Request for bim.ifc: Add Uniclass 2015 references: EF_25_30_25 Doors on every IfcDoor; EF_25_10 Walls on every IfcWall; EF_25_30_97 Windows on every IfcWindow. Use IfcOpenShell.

First a look at what the model holds.

```python
import ifcopenshell

model = ifcopenshell.open("bim.ifc")
print(model.schema)
print("classifications:", [c.Name for c in model.by_type("IfcClassification")])
for ifc_class in ("IfcDoor", "IfcRoof", "IfcStair", "IfcWall", "IfcWindow"):
    print(ifc_class, len(model.by_type(ifc_class)))
```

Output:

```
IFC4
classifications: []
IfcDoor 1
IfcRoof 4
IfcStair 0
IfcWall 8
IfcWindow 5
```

```python
import ifcopenshell
import ifcopenshell.api.classification

model = ifcopenshell.open("bim.ifc")

system = ifcopenshell.api.classification.add_classification(model, classification="Uniclass 2015")

codes = {
    "IfcDoor": ("EF_25_30_25", "Doors"),
    "IfcWall": ("EF_25_10", "Walls"),
    "IfcWindow": ("EF_25_30_97", "Windows"),
}
for ifc_class, (code, name) in codes.items():
    products = model.by_type(ifc_class)
    ifcopenshell.api.classification.add_reference(
        model, products=products, classification=system, identification=code, name=name
    )
    print(code, len(products))

model.write("bim_v2.ifc")
```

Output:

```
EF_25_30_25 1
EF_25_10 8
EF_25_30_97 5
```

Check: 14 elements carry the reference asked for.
